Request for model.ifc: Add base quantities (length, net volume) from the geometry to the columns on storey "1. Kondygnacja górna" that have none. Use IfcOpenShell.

First a look at what the model holds.

```python
import ifcopenshell
import ifcopenshell.util.element
import ifcopenshell.util.unit

model = ifcopenshell.open("model.ifc")
print(model.schema)
for unit_type in ("LENGTHUNIT", "AREAUNIT", "VOLUMEUNIT"):
    print(unit_type, ifcopenshell.util.unit.calculate_unit_scale(model, unit_type))
storey = next(s for s in model.by_type("IfcBuildingStorey") if s.Name == "1. Kondygnacja górna")
columns = [e for e in ifcopenshell.util.element.get_decomposition(storey) if e.is_a("IfcColumn")]
for e in sorted(columns, key=lambda e: e.id()):
    print(e.id(), e.is_a(), e.Name, list(ifcopenshell.util.element.get_psets(e, qtos_only=True)), sep=" | ")
```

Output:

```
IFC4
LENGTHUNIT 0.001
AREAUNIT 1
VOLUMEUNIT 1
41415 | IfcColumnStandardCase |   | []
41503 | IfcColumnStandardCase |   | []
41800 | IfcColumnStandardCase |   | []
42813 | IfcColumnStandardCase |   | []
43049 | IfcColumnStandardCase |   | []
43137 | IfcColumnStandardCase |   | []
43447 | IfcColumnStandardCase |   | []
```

```python
import ifcopenshell
import ifcopenshell.api.pset
import ifcopenshell.geom
import ifcopenshell.util.element
import ifcopenshell.util.shape
import ifcopenshell.util.unit

model = ifcopenshell.open("model.ifc")
unit_scale = ifcopenshell.util.unit.calculate_unit_scale(model)
volume_scale = ifcopenshell.util.unit.calculate_unit_scale(model, "VOLUMEUNIT")
settings = ifcopenshell.geom.settings()

storey = next(s for s in model.by_type("IfcBuildingStorey") if s.Name == "1. Kondygnacja górna")
columns = [e for e in ifcopenshell.util.element.get_decomposition(storey) if e.is_a("IfcColumn")]

for e in sorted(columns, key=lambda e: e.id()):
    if ifcopenshell.util.element.get_psets(e, qtos_only=True, should_inherit=False):
        continue
    # Geometry comes back in metres, in the element's own axes.
    shape = ifcopenshell.geom.create_shape(settings, e)
    values = {
        "Length": ifcopenshell.util.shape.get_z(shape.geometry) / unit_scale,
        "NetVolume": ifcopenshell.util.shape.get_volume(shape.geometry) / volume_scale,
    }
    qto = ifcopenshell.api.pset.add_qto(model, product=e, name="Qto_ColumnBaseQuantities")
    ifcopenshell.api.pset.edit_qto(model, qto=qto, properties=values)
    print(e.id(), {k: round(v, 3) for k, v in values.items()})

model.write("model_edited.ifc")
```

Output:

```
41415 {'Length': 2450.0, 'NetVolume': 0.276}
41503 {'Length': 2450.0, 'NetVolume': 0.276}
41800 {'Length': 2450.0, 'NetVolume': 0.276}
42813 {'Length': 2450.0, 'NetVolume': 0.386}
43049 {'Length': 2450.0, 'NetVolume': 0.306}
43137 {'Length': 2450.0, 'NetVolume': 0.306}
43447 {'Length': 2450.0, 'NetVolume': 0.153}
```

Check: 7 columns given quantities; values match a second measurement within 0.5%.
